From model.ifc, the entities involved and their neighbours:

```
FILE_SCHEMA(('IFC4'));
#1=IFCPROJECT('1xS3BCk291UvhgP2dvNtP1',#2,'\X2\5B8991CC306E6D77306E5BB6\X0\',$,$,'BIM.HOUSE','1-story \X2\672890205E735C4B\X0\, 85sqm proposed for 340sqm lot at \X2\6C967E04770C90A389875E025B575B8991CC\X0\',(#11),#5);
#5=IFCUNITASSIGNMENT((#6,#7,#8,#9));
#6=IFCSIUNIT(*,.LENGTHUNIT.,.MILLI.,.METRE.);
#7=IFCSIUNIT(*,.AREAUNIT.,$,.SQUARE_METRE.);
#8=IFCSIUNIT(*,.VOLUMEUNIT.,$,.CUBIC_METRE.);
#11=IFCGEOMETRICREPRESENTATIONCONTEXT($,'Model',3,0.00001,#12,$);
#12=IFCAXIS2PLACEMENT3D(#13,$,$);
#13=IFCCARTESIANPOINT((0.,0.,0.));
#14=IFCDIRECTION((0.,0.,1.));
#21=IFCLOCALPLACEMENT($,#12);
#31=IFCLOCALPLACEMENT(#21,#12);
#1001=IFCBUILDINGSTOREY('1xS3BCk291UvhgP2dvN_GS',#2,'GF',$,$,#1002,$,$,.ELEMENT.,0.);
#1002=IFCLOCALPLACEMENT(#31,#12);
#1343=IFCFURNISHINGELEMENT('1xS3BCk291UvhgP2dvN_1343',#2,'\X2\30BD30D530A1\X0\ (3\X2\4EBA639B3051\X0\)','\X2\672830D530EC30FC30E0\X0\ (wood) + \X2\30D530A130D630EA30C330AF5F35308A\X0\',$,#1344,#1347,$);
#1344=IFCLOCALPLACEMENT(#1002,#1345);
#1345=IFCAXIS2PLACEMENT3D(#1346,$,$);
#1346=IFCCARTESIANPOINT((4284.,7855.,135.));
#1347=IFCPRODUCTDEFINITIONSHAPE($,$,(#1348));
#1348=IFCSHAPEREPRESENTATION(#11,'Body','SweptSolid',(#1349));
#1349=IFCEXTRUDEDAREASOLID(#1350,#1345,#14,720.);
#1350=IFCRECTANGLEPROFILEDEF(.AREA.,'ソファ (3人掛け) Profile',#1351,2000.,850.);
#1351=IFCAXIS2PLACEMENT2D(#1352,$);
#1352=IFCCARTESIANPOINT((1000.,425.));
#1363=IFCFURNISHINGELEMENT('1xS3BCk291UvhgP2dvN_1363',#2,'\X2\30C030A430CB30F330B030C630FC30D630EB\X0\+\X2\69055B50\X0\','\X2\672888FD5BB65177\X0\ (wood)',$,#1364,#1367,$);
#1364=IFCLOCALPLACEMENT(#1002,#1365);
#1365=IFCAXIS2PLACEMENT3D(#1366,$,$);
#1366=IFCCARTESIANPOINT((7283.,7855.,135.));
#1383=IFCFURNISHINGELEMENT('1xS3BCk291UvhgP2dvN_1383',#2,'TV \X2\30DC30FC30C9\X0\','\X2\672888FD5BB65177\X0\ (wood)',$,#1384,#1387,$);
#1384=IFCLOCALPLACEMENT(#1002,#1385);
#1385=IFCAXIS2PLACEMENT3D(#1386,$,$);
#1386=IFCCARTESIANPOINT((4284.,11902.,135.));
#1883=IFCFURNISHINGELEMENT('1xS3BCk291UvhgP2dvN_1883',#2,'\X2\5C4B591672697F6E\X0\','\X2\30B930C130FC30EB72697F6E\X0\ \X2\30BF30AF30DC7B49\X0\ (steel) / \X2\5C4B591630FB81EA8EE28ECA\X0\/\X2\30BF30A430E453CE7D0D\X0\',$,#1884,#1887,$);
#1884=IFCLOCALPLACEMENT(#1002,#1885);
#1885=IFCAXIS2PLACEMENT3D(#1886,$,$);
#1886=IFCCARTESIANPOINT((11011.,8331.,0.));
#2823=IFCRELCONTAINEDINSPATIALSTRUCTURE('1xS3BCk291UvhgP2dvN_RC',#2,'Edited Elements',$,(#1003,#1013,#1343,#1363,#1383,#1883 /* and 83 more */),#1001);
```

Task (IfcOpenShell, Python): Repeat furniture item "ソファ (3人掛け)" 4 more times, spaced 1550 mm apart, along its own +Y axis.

```python
import ifcopenshell
import ifcopenshell.api.geometry
import ifcopenshell.api.root
import ifcopenshell.util.element
import ifcopenshell.util.placement
import ifcopenshell.util.unit

model = ifcopenshell.open("model.ifc")
unit_scale = ifcopenshell.util.unit.calculate_unit_scale(model)


def reuse_history(source, copy):
    """copy_class also copies each property set's owner history, people and application; keep the originals."""
    for rel in copy.IsDefinedBy:
        if rel.is_a("IfcRelDefinesByProperties") and (history := rel.RelatingPropertyDefinition.OwnerHistory):
            rel.RelatingPropertyDefinition.OwnerHistory = source.OwnerHistory
            ifcopenshell.util.element.remove_deep2(model, history)


source = model.by_id(1343)
base = ifcopenshell.util.placement.get_local_placement(source.ObjectPlacement)
step = base[:3, 1] * 1.55 / unit_scale

for i in range(1, 5):
    copy = ifcopenshell.api.root.copy_class(model, product=source)
    copy.Representation = ifcopenshell.util.element.copy_deep(
        model, source.Representation, exclude=["IfcGeometricRepresentationContext", "IfcRepresentationMap"]
    )
    reuse_history(source, copy)
    matrix = base.copy()
    matrix[:3, 3] += i * step
    print("added at", matrix[:3, 3].round(3) + 0.0)
    ifcopenshell.api.geometry.edit_object_placement(model, product=copy, matrix=matrix, is_si=False)

model.write("model-out.ifc")
```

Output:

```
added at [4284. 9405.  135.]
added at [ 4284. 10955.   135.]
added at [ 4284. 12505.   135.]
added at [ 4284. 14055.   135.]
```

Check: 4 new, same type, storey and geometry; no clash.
